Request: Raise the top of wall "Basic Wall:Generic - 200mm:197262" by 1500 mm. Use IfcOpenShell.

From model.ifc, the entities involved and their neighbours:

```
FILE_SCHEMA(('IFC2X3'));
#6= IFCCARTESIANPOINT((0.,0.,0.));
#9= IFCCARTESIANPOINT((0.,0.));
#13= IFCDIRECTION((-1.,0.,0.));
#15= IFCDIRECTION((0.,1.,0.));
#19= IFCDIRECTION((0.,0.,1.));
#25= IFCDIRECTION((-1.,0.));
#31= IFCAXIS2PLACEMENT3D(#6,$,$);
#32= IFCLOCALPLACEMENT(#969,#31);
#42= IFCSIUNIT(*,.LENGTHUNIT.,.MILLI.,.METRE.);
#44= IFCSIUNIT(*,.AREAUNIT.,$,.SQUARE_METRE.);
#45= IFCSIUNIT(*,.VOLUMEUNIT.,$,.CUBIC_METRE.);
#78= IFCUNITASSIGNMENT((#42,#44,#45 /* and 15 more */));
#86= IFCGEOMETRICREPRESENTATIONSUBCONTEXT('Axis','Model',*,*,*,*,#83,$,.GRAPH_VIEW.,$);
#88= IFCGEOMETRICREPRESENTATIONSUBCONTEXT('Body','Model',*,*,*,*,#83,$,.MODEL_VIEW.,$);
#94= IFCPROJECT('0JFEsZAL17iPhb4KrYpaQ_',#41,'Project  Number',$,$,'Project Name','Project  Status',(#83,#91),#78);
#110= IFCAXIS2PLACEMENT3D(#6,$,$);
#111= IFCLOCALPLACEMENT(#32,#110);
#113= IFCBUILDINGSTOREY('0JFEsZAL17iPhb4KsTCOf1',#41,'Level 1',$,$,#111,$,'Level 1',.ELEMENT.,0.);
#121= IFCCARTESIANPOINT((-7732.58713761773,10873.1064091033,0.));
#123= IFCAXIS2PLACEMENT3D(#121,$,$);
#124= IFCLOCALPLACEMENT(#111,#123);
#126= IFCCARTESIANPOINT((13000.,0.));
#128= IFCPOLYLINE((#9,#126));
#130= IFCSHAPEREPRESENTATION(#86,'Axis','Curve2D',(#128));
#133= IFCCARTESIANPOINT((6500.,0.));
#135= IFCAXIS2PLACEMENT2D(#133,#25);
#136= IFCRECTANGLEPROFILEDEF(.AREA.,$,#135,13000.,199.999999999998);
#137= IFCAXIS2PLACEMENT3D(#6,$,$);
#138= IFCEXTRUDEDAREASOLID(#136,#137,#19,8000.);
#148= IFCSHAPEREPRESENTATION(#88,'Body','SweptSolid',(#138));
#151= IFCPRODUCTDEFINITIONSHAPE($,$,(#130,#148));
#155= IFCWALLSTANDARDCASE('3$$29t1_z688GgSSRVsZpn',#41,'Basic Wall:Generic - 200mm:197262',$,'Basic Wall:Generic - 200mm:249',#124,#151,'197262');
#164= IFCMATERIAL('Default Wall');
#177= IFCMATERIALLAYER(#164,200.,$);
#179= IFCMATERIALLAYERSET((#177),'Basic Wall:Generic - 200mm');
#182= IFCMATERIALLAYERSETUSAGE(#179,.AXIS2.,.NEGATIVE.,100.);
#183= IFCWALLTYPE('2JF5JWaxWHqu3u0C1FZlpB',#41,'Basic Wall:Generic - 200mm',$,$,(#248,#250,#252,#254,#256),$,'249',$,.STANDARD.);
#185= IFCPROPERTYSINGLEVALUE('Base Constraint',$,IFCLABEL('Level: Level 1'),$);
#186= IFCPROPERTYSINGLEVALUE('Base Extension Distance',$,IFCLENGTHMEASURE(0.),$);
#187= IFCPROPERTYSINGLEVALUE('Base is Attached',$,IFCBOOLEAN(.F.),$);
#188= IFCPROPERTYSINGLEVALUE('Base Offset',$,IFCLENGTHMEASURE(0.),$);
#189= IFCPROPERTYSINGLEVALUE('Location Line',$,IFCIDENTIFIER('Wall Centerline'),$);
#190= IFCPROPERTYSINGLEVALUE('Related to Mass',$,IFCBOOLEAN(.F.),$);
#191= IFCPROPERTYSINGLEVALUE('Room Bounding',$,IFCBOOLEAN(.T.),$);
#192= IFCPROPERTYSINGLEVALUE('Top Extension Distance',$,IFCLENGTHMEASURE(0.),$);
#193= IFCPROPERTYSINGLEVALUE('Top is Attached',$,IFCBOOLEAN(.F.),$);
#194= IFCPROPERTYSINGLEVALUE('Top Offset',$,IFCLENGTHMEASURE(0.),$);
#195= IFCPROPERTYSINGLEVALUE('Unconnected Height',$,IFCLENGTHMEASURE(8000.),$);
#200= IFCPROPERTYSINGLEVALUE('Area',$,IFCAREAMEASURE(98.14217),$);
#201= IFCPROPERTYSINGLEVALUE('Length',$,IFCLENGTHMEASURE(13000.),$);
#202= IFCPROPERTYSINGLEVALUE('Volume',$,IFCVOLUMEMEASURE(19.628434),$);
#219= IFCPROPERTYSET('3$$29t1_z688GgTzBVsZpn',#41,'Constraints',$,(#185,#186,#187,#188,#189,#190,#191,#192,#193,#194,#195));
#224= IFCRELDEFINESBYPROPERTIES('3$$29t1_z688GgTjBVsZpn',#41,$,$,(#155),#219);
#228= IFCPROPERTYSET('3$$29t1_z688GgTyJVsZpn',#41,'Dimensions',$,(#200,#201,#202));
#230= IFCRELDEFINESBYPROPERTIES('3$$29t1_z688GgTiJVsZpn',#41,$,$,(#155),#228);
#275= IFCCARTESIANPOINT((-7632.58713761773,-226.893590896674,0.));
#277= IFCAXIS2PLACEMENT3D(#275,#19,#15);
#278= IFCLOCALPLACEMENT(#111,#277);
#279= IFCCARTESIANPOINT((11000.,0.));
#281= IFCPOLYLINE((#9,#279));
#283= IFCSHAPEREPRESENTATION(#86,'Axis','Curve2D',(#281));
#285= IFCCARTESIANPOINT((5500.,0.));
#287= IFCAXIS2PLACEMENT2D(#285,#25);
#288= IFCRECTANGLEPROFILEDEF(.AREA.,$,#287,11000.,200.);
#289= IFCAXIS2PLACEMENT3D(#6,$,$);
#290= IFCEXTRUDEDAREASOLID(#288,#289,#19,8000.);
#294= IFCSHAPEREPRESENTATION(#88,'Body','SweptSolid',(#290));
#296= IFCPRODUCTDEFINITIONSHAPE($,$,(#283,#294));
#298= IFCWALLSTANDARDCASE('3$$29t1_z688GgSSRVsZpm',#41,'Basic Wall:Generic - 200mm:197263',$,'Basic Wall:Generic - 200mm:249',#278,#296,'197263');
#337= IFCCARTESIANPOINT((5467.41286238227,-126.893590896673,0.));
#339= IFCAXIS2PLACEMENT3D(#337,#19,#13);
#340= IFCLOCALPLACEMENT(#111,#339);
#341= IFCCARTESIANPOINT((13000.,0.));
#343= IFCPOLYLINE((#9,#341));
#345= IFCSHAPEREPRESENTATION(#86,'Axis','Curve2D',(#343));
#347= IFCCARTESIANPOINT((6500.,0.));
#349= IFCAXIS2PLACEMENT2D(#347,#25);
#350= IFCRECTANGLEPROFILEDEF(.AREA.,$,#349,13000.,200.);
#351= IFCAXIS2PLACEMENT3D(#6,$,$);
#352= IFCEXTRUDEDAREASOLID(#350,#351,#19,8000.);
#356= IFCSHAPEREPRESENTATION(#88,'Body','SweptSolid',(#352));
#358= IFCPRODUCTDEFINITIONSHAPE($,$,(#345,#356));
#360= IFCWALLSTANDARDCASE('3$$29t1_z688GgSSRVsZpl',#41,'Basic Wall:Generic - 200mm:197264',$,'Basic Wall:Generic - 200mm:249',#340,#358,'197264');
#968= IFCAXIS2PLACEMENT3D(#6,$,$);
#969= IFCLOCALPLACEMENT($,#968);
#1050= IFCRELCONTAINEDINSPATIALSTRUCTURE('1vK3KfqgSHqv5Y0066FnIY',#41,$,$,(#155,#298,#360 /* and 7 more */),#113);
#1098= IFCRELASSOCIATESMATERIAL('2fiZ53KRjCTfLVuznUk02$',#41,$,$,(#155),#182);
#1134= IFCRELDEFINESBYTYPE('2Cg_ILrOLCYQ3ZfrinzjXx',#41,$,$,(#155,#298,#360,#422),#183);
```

```python
import ifcopenshell
import ifcopenshell.api.pset
import ifcopenshell.geom
import ifcopenshell.util.element
import ifcopenshell.util.representation
import ifcopenshell.util.shape
import ifcopenshell.util.unit

model = ifcopenshell.open("model.ifc")
unit_scale = ifcopenshell.util.unit.calculate_unit_scale(model)
area_scale = ifcopenshell.util.unit.calculate_unit_scale(model, "AREAUNIT")
volume_scale = ifcopenshell.util.unit.calculate_unit_scale(model, "VOLUMEUNIT")
settings = ifcopenshell.geom.settings()


def volume(element):
    """Net volume in cubic metres, openings subtracted."""
    shape = ifcopenshell.geom.create_shape(settings, element)
    return ifcopenshell.util.shape.get_volume(shape.geometry)


wall = model.by_guid("3$$29t1_z688GgSSRVsZpn")
before = volume(wall)

body = ifcopenshell.util.representation.get_representation(wall, "Model", "Body")
solid = body.Items[0]
old_height = solid.Depth
solid.Depth += 1.5 / unit_scale
after = volume(wall)
thickness = 0.2  # wall thickness in metres

# Update the stored height, areas and volumes.
pset = model.by_id(ifcopenshell.util.element.get_pset(wall, "Constraints", should_inherit=False)["id"])
ifcopenshell.api.pset.edit_pset(model, pset=pset, properties={
    "Unconnected Height": model.create_entity("IfcLengthMeasure", solid.Depth),
})
pset = model.by_id(ifcopenshell.util.element.get_pset(wall, "Dimensions", should_inherit=False)["id"])
ifcopenshell.api.pset.edit_pset(model, pset=pset, properties={
    "Area": model.create_entity("IfcAreaMeasure", after / thickness / area_scale),
    "Volume": model.create_entity("IfcVolumeMeasure", after / volume_scale),
})

print(f"height {old_height:g} -> {solid.Depth:g}, volume {before:.3f} -> {after:.3f} m3")

model.write("model-out.ifc")
```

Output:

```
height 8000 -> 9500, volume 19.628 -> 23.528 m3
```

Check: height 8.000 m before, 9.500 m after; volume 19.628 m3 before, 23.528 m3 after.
